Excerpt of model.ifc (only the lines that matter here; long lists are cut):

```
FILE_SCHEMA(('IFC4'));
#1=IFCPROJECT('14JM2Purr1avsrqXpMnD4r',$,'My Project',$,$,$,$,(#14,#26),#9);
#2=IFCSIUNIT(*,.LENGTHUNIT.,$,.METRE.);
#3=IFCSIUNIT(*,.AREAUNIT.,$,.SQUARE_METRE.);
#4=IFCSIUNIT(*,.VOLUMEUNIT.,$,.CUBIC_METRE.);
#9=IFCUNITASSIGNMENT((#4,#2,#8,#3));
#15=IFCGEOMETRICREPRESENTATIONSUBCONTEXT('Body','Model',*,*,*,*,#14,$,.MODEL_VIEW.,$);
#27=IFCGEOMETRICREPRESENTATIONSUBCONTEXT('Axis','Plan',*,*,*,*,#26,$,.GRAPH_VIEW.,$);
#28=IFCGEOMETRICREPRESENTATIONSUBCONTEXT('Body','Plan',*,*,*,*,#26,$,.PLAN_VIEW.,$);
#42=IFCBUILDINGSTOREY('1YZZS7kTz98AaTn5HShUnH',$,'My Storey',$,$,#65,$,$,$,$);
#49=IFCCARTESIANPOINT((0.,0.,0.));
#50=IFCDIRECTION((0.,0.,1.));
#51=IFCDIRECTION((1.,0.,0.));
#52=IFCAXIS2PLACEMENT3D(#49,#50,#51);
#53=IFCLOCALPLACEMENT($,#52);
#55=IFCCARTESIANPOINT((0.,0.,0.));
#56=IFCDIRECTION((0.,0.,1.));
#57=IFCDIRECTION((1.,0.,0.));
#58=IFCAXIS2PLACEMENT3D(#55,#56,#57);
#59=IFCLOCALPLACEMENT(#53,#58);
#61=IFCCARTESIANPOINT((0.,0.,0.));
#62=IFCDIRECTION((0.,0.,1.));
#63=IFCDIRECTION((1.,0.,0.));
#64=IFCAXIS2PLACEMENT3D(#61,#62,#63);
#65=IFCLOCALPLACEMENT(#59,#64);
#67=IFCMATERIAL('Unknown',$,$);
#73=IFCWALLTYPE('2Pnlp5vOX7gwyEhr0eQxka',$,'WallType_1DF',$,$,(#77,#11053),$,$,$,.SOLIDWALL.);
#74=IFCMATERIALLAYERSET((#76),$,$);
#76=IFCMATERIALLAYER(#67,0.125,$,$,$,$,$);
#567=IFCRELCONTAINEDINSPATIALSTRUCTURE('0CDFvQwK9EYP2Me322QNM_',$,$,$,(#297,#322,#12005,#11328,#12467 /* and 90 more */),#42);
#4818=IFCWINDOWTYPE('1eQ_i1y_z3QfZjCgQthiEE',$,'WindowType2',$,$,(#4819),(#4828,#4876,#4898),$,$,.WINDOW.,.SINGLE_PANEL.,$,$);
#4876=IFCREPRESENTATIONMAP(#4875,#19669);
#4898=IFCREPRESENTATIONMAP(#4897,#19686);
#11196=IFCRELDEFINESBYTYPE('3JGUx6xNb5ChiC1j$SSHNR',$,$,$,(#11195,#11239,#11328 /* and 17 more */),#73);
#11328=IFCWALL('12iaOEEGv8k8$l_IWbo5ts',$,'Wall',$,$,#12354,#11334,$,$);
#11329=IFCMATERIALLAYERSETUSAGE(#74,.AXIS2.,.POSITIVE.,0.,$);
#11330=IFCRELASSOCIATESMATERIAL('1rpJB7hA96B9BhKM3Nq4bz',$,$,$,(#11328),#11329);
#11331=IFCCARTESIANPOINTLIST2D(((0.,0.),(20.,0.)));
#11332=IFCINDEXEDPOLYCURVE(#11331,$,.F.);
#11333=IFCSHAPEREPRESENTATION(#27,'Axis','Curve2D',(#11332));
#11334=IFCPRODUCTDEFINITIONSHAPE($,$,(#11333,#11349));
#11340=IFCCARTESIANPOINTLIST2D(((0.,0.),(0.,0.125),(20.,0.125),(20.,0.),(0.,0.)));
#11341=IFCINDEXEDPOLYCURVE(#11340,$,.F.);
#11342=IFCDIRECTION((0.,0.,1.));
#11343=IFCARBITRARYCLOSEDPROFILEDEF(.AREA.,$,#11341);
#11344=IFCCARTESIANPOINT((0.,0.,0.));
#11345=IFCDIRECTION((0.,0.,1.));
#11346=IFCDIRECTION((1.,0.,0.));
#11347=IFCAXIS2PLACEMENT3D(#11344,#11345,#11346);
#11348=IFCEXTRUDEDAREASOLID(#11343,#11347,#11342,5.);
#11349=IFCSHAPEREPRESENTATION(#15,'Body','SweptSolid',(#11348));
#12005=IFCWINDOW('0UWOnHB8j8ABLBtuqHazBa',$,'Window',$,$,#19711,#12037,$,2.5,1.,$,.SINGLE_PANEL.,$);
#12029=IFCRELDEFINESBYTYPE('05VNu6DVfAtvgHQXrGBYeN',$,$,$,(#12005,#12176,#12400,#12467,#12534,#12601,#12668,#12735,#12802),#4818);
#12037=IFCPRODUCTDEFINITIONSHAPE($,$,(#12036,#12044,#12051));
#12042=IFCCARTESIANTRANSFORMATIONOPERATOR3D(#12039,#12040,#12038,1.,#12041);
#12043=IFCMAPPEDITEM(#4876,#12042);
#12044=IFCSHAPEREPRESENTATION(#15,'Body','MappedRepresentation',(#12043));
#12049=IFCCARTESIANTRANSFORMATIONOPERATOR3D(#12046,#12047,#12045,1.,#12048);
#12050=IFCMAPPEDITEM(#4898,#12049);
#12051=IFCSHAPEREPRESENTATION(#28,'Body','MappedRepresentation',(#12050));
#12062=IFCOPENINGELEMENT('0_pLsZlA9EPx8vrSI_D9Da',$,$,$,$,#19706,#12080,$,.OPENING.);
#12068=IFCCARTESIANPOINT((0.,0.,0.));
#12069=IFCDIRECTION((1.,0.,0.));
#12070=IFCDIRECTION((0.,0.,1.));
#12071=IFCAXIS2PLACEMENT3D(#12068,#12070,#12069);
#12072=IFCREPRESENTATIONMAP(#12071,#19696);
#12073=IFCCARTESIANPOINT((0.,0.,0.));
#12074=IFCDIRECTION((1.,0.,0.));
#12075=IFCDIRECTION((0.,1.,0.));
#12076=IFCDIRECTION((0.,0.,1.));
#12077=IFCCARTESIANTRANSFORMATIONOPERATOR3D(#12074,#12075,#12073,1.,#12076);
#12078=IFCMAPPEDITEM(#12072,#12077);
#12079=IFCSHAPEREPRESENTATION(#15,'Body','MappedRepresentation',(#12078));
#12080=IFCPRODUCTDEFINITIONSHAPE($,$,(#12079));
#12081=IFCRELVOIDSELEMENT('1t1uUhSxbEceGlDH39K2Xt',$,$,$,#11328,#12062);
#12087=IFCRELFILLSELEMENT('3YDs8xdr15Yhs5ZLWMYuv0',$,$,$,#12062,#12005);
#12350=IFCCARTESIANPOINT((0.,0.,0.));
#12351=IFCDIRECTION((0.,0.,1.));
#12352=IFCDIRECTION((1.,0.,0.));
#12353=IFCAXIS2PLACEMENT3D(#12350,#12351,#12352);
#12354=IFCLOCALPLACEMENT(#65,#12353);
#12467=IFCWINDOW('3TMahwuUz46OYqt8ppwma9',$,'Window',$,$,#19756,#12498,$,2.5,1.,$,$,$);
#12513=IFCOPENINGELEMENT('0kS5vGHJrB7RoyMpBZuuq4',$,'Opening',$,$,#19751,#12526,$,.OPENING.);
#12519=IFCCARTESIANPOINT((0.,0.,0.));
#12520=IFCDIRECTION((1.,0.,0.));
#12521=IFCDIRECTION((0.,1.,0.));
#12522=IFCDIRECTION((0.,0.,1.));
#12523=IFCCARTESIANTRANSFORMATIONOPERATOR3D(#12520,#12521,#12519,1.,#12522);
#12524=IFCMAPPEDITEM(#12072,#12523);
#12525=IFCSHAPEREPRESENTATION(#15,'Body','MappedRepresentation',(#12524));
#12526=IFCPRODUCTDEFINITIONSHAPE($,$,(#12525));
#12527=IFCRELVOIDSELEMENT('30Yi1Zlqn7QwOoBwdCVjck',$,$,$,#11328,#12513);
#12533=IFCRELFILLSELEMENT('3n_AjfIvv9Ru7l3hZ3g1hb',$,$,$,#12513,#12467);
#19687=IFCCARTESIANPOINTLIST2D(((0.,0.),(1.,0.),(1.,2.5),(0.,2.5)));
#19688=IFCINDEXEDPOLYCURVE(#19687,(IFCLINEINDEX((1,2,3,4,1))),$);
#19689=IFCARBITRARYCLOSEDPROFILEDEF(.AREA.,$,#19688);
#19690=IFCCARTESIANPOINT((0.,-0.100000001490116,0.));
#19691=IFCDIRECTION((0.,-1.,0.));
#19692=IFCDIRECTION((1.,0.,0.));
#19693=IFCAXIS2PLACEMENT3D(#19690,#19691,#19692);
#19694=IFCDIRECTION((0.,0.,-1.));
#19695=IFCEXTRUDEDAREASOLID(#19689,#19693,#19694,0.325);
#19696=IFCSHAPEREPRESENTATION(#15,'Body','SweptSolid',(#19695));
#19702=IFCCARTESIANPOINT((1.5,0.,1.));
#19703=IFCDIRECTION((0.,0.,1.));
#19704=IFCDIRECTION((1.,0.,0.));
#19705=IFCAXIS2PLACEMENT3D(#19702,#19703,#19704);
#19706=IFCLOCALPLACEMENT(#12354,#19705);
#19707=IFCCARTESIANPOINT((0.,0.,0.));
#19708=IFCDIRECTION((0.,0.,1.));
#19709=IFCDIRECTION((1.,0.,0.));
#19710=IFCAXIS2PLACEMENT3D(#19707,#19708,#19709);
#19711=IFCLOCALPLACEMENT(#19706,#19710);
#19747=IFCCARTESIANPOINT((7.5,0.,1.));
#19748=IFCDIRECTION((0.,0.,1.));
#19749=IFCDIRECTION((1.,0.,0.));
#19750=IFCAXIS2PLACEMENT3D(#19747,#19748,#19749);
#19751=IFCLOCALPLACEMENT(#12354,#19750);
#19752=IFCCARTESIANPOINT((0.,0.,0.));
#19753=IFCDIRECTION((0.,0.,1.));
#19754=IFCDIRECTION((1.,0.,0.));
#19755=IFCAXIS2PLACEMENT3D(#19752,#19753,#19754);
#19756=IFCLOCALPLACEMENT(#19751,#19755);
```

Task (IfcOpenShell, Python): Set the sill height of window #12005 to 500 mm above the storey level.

```python
import numpy as np
import ifcopenshell
import ifcopenshell.api.geometry
import ifcopenshell.geom
import ifcopenshell.util.element
import ifcopenshell.util.placement
import ifcopenshell.util.shape
import ifcopenshell.util.unit

model = ifcopenshell.open("model.ifc")
unit_scale = ifcopenshell.util.unit.calculate_unit_scale(model)

window = model.by_guid("0UWOnHB8j8ABLBtuqHazBa")
opening = window.FillsVoids[0].RelatingOpeningElement
storey = ifcopenshell.util.element.get_container(window, ifc_class="IfcBuildingStorey")
level = ifcopenshell.util.placement.get_local_placement(storey.ObjectPlacement)[2, 3]

# The opening's origin need not be at the sill, so measure its lowest point.
shape = ifcopenshell.geom.create_shape(ifcopenshell.geom.settings(), opening)
bottom = ifcopenshell.util.shape.get_shape_bottom_elevation(shape, shape.geometry) / unit_scale
dz = level + 0.5 - bottom

shift = np.array([0.0, 0.0, dz])
# The window is placed relative to its opening, so it follows when the opening moves.
matrix = ifcopenshell.util.placement.get_local_placement(opening.ObjectPlacement)
matrix[:3, 3] += shift
ifcopenshell.api.geometry.edit_object_placement(
    model, product=opening, matrix=matrix, is_si=False, should_transform_children=True
)

print(f"moved by {dz * unit_scale:+.3f} m")

model.write("model_rev.ifc")
```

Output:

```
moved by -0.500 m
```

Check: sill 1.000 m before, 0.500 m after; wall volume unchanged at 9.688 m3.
